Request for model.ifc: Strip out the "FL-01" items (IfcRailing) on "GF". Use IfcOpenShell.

First a look at what the model holds.

```python
import ifcopenshell
import ifcopenshell.util.element

model = ifcopenshell.open("model.ifc")
print(model.schema)
storey = next(s for s in model.by_type("IfcBuildingStorey") if s.Name == "GF")
railings = [e for e in ifcopenshell.util.element.get_decomposition(storey) if e.is_a("IfcRailing")]
seen = {}
for e in railings:
    element_type = ifcopenshell.util.element.get_type(e)
    name = element_type.Name if element_type not in (None, e) else None
    seen[name] = seen.get(name, 0) + 1
for name, count in sorted(seen.items(), key=str):
    print(count, "x", name)
```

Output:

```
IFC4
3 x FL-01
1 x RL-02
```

```python
import ifcopenshell
import ifcopenshell.api.root
import ifcopenshell.util.element

model = ifcopenshell.open("model.ifc")

storey = next(s for s in model.by_type("IfcBuildingStorey") if s.Name == "GF")
railings = [e for e in ifcopenshell.util.element.get_decomposition(storey) if e.is_a("IfcRailing")]
targets = [e for e in railings if (t := ifcopenshell.util.element.get_type(e)) not in (None, e) and t.Name == "FL-01"]

for e in targets:
    ifcopenshell.api.root.remove_product(model, product=e)
print(len(targets), "removed")

model.write("model-out.ifc")
```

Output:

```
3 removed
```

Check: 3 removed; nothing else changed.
